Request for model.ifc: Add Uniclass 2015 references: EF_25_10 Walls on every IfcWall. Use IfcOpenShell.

First a look at what the model holds.

```python
import ifcopenshell

model = ifcopenshell.open("model.ifc")
print(model.schema)
print("classifications:", [c.Name for c in model.by_type("IfcClassification")])
for ifc_class in ("IfcDoor", "IfcRoof", "IfcStair", "IfcWall", "IfcWindow"):
    print(ifc_class, len(model.by_type(ifc_class)))
```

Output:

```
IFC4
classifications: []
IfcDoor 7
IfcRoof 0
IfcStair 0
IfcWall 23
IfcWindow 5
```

```python
import ifcopenshell
import ifcopenshell.api.classification

model = ifcopenshell.open("model.ifc")

system = ifcopenshell.api.classification.add_classification(model, classification="Uniclass 2015")

codes = {
    "IfcWall": ("EF_25_10", "Walls"),
}
for ifc_class, (code, name) in codes.items():
    products = model.by_type(ifc_class)
    ifcopenshell.api.classification.add_reference(
        model, products=products, classification=system, identification=code, name=name
    )
    print(code, len(products))

model.write("model_rev.ifc")
```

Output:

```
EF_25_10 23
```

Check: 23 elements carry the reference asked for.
